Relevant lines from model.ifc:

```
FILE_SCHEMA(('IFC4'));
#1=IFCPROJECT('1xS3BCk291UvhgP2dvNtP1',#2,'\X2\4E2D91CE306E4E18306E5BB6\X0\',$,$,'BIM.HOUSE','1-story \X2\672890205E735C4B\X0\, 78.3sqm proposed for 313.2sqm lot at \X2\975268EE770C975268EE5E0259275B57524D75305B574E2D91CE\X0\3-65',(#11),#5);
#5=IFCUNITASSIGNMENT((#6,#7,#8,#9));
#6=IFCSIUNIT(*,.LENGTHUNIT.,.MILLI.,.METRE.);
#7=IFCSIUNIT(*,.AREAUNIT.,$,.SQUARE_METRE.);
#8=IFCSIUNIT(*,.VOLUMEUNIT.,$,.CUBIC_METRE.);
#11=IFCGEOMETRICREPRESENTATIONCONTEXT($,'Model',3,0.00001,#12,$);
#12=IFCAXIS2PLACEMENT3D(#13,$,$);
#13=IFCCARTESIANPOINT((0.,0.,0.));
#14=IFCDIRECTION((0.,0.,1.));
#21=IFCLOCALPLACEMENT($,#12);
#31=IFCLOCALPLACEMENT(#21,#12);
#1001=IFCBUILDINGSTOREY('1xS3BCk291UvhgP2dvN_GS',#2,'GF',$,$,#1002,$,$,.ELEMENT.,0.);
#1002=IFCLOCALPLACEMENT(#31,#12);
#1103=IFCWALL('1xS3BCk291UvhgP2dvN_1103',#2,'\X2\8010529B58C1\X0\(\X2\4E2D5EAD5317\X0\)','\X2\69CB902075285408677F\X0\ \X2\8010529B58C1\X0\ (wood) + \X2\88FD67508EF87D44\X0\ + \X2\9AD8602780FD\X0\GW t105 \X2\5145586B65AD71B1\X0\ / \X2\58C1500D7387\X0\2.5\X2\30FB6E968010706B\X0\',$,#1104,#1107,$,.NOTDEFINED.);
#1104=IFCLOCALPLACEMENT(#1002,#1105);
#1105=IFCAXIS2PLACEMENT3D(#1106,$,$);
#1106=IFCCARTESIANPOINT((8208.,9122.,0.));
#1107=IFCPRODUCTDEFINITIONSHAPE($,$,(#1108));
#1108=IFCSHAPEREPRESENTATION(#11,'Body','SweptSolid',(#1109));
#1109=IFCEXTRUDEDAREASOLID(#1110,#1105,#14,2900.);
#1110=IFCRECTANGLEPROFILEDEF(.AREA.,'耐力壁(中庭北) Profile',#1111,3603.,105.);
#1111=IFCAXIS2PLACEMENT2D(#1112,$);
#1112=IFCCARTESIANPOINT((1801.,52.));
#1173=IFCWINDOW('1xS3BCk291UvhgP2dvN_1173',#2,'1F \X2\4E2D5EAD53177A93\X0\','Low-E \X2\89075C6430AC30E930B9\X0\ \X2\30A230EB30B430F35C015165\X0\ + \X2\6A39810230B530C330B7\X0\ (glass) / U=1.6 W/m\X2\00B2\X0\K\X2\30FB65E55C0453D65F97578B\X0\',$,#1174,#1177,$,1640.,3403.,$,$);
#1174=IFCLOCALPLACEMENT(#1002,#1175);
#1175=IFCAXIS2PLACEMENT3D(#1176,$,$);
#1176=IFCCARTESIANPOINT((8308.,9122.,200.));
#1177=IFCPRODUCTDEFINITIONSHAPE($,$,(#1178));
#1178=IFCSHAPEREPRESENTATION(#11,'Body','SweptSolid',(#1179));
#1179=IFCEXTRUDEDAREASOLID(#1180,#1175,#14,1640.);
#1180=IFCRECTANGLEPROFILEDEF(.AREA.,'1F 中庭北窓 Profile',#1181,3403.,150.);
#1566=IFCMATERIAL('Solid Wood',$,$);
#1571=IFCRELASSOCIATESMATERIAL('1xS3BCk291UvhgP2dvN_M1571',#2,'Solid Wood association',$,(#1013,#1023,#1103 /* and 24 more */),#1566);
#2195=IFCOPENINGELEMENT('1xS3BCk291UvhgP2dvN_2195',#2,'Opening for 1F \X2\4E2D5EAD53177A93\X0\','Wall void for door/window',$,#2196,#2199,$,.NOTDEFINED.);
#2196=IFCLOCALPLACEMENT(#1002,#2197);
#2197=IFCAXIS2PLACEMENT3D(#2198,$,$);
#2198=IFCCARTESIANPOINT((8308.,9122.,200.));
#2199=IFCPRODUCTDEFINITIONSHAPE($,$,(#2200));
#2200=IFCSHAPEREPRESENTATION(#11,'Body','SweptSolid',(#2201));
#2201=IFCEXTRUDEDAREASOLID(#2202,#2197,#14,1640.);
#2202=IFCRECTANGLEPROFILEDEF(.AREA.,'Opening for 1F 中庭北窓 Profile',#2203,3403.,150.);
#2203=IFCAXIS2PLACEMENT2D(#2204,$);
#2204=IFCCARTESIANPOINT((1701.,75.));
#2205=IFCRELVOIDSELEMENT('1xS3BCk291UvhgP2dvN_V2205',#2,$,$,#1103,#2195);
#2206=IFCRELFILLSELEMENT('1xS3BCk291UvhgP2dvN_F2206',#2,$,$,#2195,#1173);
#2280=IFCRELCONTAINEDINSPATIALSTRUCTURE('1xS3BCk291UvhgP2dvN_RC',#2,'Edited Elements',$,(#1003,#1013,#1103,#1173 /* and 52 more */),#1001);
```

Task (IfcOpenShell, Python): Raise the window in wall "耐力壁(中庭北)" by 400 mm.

```python
import numpy as np
import ifcopenshell
import ifcopenshell.api.geometry
import ifcopenshell.util.placement
import ifcopenshell.util.unit

model = ifcopenshell.open("model.ifc")
unit_scale = ifcopenshell.util.unit.calculate_unit_scale(model)

window = model.by_guid("1xS3BCk291UvhgP2dvN_1173")
opening = window.FillsVoids[0].RelatingOpeningElement
dz = 400.0

shift = np.array([0.0, 0.0, dz])
# The window is not placed relative to its opening, so move both.
for product in (opening, window):
    matrix = ifcopenshell.util.placement.get_local_placement(product.ObjectPlacement)
    matrix[:3, 3] += shift
    ifcopenshell.api.geometry.edit_object_placement(model, product=product, matrix=matrix, is_si=False)

print(f"moved by {dz * unit_scale:+.3f} m")

model.write("model-out.ifc")
```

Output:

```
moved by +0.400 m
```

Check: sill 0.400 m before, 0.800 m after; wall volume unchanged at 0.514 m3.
